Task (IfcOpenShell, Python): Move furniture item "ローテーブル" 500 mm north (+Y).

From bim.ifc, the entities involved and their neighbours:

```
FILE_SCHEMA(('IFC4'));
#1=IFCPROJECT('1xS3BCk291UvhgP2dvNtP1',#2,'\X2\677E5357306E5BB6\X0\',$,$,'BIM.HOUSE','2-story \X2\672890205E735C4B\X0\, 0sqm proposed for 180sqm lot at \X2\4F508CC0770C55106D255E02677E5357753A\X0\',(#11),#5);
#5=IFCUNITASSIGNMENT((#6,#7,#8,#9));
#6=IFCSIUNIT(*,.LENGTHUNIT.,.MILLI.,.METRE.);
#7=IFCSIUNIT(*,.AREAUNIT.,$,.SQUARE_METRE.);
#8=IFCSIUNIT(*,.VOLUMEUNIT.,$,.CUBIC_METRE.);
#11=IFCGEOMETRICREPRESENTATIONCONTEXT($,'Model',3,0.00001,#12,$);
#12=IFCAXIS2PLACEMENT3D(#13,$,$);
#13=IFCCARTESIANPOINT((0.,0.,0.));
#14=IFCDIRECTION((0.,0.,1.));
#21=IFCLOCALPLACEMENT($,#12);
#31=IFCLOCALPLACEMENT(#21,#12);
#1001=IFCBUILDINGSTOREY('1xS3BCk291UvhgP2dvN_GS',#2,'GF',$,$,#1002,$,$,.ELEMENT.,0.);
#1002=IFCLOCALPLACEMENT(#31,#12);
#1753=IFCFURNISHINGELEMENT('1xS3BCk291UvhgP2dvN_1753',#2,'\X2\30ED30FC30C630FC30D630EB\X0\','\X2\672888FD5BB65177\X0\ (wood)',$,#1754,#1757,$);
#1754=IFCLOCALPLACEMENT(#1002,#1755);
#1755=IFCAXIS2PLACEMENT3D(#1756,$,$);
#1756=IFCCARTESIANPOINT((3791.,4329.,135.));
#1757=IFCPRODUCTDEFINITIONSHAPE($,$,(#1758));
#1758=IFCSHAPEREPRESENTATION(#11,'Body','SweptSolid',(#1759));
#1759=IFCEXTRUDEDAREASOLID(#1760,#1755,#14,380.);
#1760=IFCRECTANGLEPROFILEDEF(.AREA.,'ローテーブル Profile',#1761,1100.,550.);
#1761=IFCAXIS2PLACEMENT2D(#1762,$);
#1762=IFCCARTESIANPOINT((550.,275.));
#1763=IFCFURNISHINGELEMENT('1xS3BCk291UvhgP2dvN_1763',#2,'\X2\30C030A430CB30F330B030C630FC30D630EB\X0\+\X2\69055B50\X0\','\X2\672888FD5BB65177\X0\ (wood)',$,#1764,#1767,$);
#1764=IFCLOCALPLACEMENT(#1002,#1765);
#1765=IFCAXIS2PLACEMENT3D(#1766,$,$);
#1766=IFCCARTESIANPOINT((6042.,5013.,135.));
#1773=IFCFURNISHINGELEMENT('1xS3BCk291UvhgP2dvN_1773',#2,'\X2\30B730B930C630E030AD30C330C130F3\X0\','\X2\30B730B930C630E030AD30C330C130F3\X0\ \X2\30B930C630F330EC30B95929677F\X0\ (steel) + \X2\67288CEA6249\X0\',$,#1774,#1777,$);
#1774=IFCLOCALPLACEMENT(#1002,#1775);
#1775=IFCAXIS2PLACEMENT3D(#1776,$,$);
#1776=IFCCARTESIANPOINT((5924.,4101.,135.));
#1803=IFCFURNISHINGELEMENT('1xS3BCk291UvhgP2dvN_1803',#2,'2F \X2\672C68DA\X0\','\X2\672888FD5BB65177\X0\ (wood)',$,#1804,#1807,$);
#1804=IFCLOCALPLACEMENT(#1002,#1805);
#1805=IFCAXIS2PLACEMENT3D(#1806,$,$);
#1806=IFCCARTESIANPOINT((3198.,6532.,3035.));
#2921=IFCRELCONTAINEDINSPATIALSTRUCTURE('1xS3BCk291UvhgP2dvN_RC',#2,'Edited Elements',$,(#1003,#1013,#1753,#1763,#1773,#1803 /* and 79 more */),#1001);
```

```python
import ifcopenshell
import ifcopenshell.api.geometry
import ifcopenshell.util.placement

model = ifcopenshell.open("bim.ifc")

item = model.by_id(1753)
matrix = ifcopenshell.util.placement.get_local_placement(item.ObjectPlacement)
matrix[1, 3] += 500.0
ifcopenshell.api.geometry.edit_object_placement(model, product=item, matrix=matrix, is_si=False)

print(ifcopenshell.util.placement.get_local_placement(item.ObjectPlacement).round(3) + 0.0)

model.write("bim_rev.ifc")
```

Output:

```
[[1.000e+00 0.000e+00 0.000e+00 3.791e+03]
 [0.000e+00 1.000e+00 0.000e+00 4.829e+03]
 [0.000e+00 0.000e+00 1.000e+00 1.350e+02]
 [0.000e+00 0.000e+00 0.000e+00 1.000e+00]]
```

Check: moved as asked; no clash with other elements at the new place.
